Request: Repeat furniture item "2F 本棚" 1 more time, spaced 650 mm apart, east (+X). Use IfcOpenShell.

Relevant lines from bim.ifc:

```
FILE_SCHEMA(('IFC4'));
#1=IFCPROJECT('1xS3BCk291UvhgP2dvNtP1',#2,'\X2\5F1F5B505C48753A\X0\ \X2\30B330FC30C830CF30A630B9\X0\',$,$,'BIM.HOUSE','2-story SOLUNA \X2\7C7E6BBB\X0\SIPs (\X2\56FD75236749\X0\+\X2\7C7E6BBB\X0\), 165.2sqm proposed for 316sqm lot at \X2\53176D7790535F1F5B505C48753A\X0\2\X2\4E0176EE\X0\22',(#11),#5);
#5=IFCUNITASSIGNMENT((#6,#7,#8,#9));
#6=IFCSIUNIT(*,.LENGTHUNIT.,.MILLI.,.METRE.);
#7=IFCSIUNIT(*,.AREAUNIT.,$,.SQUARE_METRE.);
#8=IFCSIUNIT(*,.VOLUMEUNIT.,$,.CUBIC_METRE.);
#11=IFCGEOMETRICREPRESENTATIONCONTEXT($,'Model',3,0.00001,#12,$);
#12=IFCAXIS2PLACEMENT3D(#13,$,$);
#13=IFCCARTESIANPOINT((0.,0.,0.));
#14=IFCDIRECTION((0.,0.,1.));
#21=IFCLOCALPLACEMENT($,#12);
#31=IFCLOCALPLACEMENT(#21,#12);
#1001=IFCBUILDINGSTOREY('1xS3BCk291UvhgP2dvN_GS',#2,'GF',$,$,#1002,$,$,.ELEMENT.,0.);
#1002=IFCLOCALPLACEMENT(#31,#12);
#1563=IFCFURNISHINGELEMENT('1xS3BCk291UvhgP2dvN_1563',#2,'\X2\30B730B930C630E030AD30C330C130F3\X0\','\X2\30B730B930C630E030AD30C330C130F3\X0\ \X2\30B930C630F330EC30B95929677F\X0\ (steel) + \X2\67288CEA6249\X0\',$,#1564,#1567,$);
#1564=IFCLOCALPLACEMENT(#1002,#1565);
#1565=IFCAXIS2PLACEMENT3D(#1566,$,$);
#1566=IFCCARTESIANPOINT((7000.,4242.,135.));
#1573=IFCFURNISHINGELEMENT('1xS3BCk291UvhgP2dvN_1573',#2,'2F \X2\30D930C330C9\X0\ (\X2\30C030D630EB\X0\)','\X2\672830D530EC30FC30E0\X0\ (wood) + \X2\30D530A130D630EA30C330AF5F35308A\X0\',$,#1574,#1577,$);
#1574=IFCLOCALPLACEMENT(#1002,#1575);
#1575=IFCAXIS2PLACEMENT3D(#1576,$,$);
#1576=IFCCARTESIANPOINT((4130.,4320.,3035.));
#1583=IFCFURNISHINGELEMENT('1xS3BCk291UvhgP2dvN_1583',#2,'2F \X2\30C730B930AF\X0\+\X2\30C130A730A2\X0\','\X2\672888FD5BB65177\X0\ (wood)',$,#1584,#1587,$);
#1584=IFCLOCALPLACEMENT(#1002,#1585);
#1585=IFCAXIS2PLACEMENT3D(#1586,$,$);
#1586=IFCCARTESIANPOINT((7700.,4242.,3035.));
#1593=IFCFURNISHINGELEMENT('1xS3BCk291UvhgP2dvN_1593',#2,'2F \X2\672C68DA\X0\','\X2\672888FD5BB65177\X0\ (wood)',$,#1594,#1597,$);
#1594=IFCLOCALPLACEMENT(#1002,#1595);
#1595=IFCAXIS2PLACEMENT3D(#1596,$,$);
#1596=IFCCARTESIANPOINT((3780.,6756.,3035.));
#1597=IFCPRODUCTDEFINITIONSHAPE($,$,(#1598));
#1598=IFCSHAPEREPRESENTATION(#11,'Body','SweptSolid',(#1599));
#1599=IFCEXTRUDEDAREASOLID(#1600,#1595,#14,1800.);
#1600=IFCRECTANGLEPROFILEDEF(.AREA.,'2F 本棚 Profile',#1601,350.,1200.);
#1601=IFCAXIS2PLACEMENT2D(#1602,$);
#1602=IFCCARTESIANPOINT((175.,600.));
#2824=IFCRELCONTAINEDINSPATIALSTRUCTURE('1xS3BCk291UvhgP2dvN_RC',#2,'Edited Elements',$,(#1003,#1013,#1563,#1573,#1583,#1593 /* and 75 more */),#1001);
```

```python
import numpy as np
import ifcopenshell
import ifcopenshell.api.geometry
import ifcopenshell.api.root
import ifcopenshell.util.element
import ifcopenshell.util.placement

model = ifcopenshell.open("bim.ifc")


def reuse_history(source, copy):
    """copy_class also copies each property set's owner history, people and application; keep the originals."""
    for rel in copy.IsDefinedBy:
        if rel.is_a("IfcRelDefinesByProperties") and (history := rel.RelatingPropertyDefinition.OwnerHistory):
            rel.RelatingPropertyDefinition.OwnerHistory = source.OwnerHistory
            ifcopenshell.util.element.remove_deep2(model, history)


source = model.by_id(1593)
base = ifcopenshell.util.placement.get_local_placement(source.ObjectPlacement)
step = np.array([1.0, 0.0, 0.0]) * 650.0

for i in range(1, 2):
    copy = ifcopenshell.api.root.copy_class(model, product=source)
    copy.Representation = ifcopenshell.util.element.copy_deep(
        model, source.Representation, exclude=["IfcGeometricRepresentationContext", "IfcRepresentationMap"]
    )
    reuse_history(source, copy)
    matrix = base.copy()
    matrix[:3, 3] += i * step
    print("added at", matrix[:3, 3].round(3) + 0.0)
    ifcopenshell.api.geometry.edit_object_placement(model, product=copy, matrix=matrix, is_si=False)

model.write("bim_edited.ifc")
```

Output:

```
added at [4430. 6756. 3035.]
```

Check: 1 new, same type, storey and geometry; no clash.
